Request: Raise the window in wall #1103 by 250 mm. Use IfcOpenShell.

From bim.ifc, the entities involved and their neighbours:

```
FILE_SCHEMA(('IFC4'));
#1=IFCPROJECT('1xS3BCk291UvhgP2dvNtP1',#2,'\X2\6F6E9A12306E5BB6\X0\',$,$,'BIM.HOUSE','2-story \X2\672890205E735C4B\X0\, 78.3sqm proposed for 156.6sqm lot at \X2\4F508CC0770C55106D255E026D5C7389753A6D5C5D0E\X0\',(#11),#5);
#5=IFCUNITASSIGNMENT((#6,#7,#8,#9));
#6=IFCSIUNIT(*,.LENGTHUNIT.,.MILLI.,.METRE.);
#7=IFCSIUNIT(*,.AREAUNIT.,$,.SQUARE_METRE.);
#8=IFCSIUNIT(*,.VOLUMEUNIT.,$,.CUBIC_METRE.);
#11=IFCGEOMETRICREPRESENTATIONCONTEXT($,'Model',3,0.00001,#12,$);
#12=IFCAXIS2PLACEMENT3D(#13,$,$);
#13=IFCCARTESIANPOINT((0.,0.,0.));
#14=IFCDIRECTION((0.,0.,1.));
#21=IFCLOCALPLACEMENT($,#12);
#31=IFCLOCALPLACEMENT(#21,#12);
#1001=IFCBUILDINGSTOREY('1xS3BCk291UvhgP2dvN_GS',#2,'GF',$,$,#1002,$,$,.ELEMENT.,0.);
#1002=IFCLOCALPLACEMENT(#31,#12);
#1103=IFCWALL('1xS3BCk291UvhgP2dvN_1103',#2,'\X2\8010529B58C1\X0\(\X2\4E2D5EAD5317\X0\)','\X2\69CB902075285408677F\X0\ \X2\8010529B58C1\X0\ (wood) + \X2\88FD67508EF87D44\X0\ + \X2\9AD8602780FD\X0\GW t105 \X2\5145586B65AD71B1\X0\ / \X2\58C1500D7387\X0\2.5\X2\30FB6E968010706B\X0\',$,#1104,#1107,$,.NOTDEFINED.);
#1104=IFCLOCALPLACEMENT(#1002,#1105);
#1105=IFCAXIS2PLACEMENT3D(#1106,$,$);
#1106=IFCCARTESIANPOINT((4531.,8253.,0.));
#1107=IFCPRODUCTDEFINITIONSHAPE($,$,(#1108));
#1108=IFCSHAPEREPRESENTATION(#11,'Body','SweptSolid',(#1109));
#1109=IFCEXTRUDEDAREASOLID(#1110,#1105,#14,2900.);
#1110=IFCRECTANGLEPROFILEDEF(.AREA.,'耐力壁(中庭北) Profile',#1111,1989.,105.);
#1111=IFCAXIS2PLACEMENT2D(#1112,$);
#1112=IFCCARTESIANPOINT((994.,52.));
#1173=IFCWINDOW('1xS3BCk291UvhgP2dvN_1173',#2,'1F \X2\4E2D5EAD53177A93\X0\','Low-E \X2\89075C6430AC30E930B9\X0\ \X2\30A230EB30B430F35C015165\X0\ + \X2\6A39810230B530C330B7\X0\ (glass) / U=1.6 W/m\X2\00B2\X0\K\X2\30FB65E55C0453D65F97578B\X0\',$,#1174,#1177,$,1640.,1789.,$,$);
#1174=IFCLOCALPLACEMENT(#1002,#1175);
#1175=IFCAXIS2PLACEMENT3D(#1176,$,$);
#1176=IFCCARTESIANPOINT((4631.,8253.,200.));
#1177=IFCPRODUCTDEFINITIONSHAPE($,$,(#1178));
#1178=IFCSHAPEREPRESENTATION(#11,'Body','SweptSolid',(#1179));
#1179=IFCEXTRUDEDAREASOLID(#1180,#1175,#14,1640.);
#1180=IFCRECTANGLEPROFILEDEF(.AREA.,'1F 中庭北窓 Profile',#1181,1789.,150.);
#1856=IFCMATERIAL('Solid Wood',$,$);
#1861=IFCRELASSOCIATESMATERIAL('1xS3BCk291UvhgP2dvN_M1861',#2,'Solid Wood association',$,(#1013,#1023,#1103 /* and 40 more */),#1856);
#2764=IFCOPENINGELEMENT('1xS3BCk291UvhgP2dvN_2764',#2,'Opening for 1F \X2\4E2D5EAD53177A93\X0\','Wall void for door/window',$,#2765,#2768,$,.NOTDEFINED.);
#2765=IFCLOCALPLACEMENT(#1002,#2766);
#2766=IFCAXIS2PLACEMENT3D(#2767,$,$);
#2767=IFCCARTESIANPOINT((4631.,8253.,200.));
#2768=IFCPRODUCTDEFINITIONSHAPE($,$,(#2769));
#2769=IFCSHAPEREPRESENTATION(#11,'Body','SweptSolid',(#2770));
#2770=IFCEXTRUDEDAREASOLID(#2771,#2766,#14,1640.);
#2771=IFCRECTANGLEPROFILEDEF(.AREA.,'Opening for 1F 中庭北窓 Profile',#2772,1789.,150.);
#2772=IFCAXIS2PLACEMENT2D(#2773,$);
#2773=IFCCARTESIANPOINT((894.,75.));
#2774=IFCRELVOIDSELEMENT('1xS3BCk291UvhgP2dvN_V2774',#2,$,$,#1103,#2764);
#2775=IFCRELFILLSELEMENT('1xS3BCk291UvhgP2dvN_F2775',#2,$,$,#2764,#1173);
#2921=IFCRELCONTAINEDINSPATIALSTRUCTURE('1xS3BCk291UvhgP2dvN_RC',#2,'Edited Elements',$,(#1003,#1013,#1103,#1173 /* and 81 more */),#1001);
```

```python
import numpy as np
import ifcopenshell
import ifcopenshell.api.geometry
import ifcopenshell.util.placement
import ifcopenshell.util.unit

model = ifcopenshell.open("bim.ifc")
unit_scale = ifcopenshell.util.unit.calculate_unit_scale(model)

window = model.by_guid("1xS3BCk291UvhgP2dvN_1173")
opening = window.FillsVoids[0].RelatingOpeningElement
dz = 250.0

shift = np.array([0.0, 0.0, dz])
# The window is not placed relative to its opening, so move both.
for product in (opening, window):
    matrix = ifcopenshell.util.placement.get_local_placement(product.ObjectPlacement)
    matrix[:3, 3] += shift
    ifcopenshell.api.geometry.edit_object_placement(model, product=product, matrix=matrix, is_si=False)

print(f"moved by {dz * unit_scale:+.3f} m")

model.write("bim_updated.ifc")
```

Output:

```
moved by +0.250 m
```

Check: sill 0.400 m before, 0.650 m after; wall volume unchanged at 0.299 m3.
